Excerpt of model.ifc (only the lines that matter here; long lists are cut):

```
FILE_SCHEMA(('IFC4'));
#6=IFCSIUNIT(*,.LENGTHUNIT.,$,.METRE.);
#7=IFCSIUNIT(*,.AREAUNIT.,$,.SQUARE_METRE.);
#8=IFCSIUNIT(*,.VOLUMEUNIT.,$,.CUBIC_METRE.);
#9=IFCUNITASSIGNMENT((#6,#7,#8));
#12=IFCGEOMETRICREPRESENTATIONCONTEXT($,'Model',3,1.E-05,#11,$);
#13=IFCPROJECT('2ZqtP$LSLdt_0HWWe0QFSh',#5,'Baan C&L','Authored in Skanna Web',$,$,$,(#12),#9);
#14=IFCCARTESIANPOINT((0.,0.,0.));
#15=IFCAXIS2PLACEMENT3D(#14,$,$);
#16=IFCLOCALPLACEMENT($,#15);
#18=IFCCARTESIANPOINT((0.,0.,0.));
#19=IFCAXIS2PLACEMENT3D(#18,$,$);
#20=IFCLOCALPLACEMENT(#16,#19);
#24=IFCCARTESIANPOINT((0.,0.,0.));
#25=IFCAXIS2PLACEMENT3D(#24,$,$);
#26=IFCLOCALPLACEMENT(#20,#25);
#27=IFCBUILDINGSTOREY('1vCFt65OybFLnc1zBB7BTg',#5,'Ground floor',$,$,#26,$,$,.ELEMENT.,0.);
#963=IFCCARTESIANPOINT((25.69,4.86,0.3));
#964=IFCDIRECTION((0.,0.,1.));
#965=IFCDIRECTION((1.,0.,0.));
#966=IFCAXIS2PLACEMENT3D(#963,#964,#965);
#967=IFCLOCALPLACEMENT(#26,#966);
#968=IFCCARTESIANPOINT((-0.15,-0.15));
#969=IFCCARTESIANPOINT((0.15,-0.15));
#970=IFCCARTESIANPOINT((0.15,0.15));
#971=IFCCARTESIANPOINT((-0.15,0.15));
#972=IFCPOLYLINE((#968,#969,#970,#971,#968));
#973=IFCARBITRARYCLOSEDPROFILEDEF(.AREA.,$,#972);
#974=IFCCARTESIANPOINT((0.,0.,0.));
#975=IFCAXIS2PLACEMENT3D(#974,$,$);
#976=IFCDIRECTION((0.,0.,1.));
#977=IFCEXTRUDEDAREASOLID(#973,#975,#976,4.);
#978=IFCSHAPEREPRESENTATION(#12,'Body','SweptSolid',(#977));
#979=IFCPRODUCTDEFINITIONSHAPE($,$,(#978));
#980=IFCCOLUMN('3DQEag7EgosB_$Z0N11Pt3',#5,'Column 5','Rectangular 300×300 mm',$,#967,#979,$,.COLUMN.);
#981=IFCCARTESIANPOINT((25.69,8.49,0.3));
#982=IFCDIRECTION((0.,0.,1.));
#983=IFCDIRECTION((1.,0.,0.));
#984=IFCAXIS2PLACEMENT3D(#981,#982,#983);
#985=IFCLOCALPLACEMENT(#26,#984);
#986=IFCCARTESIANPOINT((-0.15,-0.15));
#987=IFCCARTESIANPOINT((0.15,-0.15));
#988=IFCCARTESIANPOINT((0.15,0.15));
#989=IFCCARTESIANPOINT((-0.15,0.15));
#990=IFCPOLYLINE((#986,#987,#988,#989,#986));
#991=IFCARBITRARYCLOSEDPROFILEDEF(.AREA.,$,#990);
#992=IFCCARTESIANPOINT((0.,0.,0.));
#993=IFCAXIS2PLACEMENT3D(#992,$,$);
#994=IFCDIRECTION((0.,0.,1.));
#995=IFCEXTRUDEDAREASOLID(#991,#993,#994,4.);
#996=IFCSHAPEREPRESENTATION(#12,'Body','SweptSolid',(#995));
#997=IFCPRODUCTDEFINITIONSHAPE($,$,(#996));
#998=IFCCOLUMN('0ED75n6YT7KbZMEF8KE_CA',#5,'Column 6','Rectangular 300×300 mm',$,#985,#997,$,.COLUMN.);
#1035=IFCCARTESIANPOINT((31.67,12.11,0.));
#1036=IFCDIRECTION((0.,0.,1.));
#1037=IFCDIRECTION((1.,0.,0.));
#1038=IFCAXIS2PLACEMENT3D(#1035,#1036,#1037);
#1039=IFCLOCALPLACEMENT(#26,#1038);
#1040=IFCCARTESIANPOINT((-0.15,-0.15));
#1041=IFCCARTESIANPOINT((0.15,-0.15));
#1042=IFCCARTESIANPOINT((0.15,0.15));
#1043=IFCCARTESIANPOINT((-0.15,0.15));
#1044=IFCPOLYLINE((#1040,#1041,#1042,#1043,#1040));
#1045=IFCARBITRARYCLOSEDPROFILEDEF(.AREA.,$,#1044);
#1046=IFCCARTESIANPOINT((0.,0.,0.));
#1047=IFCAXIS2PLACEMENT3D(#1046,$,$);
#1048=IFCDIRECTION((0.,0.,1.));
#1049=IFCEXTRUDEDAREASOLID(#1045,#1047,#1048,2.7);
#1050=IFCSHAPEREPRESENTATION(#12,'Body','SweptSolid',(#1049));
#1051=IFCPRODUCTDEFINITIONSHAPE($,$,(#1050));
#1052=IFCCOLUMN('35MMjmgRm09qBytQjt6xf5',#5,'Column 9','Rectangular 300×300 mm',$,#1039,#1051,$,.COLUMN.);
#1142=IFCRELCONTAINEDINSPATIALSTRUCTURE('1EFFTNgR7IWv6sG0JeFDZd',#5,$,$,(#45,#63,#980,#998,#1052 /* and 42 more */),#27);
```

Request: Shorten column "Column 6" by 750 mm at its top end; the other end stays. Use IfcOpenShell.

```python
import ifcopenshell

model = ifcopenshell.open("model.ifc")

member = model.by_guid("0ED75n6YT7KbZMEF8KE_CA")
change = -0.75

# The extrusion runs towards the end named, so only its depth changes.
body = next(r for r in member.Representation.Representations if r.RepresentationIdentifier == "Body")
solid = body.Items[0]
old_length = solid.Depth
solid.Depth += change

print(f"length {old_length:g} -> {solid.Depth:g}")

model.write("model_updated.ifc")
```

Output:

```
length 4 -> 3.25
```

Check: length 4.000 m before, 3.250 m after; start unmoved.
